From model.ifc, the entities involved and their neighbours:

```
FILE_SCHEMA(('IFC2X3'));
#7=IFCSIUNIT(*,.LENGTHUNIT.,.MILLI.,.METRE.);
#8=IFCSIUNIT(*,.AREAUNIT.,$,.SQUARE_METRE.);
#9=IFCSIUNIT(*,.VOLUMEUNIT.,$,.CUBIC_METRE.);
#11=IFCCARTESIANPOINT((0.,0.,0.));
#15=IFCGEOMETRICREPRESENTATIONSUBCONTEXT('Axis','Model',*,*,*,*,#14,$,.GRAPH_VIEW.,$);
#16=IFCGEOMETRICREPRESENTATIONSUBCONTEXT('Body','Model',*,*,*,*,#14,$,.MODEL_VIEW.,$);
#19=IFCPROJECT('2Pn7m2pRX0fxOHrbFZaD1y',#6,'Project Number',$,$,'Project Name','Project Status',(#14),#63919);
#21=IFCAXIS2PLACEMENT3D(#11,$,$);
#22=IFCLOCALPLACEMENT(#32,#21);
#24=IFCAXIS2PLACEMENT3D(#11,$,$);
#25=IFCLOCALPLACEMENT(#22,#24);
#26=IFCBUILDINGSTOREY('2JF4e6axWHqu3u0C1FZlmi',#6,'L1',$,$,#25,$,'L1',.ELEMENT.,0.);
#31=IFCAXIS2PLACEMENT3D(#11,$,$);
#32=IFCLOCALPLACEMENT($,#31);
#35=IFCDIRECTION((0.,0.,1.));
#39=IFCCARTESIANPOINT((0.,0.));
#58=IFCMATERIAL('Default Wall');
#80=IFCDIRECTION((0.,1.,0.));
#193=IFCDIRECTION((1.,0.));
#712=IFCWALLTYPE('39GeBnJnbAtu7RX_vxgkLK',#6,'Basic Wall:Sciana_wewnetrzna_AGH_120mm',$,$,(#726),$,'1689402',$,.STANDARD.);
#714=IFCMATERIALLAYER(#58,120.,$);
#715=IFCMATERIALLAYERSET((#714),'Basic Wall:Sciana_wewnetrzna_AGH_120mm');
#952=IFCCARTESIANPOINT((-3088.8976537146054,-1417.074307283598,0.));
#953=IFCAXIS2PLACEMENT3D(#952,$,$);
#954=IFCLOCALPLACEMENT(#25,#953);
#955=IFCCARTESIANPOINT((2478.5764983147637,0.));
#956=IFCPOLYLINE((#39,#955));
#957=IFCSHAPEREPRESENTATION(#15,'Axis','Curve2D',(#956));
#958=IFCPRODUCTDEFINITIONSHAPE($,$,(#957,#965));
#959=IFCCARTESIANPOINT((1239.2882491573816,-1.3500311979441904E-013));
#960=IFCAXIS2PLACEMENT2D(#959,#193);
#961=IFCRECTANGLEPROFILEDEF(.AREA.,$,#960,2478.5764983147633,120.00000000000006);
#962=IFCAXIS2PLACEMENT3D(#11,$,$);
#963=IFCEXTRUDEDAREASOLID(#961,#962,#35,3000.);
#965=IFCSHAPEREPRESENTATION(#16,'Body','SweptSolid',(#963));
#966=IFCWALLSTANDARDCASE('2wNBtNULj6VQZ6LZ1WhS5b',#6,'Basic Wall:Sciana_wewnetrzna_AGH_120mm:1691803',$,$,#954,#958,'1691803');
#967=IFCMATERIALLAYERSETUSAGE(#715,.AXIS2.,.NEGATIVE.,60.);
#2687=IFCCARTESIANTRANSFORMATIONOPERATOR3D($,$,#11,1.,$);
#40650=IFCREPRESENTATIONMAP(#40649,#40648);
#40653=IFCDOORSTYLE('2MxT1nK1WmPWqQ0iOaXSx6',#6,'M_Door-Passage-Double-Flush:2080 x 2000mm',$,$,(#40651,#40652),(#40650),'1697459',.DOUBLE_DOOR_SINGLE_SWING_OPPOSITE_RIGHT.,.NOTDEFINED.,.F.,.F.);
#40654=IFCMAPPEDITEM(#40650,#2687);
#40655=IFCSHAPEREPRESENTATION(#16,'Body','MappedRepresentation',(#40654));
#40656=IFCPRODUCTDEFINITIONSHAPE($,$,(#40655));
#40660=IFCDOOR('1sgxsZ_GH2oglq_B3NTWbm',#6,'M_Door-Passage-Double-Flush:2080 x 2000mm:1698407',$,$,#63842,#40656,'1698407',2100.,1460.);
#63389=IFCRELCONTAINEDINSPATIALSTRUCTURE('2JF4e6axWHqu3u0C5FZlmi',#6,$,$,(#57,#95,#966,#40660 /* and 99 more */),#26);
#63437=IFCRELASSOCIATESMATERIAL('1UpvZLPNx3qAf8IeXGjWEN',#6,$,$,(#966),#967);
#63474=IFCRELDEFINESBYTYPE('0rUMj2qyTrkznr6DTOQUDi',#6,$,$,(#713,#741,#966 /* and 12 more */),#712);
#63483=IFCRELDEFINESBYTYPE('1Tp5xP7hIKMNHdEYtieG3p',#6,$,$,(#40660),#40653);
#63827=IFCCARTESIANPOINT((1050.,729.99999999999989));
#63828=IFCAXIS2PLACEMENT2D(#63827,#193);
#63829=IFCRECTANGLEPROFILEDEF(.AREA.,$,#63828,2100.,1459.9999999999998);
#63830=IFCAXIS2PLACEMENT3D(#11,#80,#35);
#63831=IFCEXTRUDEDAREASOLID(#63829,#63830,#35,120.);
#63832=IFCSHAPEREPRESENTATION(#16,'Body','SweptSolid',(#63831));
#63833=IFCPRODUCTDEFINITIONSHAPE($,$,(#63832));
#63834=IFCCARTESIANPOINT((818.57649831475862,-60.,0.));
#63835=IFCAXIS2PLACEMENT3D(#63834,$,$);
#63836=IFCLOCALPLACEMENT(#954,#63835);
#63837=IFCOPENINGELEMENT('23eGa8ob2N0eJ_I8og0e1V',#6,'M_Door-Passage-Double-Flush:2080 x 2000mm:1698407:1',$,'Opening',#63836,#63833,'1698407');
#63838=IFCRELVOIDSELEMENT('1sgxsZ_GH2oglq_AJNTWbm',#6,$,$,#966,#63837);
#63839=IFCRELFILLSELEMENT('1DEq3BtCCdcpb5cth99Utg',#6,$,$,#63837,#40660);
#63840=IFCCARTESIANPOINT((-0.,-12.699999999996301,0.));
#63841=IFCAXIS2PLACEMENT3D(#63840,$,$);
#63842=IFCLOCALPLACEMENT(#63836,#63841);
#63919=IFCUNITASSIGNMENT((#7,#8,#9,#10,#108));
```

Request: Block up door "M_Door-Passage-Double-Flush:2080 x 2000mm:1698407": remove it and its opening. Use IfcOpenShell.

```python
import ifcopenshell
import ifcopenshell.api.feature
import ifcopenshell.api.root
import ifcopenshell.geom
import ifcopenshell.util.shape

model = ifcopenshell.open("model.ifc")
settings = ifcopenshell.geom.settings()


def volume(element):
    """Net volume in cubic metres, openings subtracted."""
    shape = ifcopenshell.geom.create_shape(settings, element)
    return ifcopenshell.util.shape.get_volume(shape.geometry)


door = model.by_guid("1sgxsZ_GH2oglq_B3NTWbm")
opening = door.FillsVoids[0].RelatingOpeningElement
wall = opening.VoidsElements[0].RelatingBuildingElement
before = volume(wall)

ifcopenshell.api.root.remove_product(model, product=door)
ifcopenshell.api.feature.remove_feature(model, feature=opening)

after = volume(wall)

print(f"wall volume {before:.3f} -> {after:.3f} m3")

model.write("model_rev.ifc")
```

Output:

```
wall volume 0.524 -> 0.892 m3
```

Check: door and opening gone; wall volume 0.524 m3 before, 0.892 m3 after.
